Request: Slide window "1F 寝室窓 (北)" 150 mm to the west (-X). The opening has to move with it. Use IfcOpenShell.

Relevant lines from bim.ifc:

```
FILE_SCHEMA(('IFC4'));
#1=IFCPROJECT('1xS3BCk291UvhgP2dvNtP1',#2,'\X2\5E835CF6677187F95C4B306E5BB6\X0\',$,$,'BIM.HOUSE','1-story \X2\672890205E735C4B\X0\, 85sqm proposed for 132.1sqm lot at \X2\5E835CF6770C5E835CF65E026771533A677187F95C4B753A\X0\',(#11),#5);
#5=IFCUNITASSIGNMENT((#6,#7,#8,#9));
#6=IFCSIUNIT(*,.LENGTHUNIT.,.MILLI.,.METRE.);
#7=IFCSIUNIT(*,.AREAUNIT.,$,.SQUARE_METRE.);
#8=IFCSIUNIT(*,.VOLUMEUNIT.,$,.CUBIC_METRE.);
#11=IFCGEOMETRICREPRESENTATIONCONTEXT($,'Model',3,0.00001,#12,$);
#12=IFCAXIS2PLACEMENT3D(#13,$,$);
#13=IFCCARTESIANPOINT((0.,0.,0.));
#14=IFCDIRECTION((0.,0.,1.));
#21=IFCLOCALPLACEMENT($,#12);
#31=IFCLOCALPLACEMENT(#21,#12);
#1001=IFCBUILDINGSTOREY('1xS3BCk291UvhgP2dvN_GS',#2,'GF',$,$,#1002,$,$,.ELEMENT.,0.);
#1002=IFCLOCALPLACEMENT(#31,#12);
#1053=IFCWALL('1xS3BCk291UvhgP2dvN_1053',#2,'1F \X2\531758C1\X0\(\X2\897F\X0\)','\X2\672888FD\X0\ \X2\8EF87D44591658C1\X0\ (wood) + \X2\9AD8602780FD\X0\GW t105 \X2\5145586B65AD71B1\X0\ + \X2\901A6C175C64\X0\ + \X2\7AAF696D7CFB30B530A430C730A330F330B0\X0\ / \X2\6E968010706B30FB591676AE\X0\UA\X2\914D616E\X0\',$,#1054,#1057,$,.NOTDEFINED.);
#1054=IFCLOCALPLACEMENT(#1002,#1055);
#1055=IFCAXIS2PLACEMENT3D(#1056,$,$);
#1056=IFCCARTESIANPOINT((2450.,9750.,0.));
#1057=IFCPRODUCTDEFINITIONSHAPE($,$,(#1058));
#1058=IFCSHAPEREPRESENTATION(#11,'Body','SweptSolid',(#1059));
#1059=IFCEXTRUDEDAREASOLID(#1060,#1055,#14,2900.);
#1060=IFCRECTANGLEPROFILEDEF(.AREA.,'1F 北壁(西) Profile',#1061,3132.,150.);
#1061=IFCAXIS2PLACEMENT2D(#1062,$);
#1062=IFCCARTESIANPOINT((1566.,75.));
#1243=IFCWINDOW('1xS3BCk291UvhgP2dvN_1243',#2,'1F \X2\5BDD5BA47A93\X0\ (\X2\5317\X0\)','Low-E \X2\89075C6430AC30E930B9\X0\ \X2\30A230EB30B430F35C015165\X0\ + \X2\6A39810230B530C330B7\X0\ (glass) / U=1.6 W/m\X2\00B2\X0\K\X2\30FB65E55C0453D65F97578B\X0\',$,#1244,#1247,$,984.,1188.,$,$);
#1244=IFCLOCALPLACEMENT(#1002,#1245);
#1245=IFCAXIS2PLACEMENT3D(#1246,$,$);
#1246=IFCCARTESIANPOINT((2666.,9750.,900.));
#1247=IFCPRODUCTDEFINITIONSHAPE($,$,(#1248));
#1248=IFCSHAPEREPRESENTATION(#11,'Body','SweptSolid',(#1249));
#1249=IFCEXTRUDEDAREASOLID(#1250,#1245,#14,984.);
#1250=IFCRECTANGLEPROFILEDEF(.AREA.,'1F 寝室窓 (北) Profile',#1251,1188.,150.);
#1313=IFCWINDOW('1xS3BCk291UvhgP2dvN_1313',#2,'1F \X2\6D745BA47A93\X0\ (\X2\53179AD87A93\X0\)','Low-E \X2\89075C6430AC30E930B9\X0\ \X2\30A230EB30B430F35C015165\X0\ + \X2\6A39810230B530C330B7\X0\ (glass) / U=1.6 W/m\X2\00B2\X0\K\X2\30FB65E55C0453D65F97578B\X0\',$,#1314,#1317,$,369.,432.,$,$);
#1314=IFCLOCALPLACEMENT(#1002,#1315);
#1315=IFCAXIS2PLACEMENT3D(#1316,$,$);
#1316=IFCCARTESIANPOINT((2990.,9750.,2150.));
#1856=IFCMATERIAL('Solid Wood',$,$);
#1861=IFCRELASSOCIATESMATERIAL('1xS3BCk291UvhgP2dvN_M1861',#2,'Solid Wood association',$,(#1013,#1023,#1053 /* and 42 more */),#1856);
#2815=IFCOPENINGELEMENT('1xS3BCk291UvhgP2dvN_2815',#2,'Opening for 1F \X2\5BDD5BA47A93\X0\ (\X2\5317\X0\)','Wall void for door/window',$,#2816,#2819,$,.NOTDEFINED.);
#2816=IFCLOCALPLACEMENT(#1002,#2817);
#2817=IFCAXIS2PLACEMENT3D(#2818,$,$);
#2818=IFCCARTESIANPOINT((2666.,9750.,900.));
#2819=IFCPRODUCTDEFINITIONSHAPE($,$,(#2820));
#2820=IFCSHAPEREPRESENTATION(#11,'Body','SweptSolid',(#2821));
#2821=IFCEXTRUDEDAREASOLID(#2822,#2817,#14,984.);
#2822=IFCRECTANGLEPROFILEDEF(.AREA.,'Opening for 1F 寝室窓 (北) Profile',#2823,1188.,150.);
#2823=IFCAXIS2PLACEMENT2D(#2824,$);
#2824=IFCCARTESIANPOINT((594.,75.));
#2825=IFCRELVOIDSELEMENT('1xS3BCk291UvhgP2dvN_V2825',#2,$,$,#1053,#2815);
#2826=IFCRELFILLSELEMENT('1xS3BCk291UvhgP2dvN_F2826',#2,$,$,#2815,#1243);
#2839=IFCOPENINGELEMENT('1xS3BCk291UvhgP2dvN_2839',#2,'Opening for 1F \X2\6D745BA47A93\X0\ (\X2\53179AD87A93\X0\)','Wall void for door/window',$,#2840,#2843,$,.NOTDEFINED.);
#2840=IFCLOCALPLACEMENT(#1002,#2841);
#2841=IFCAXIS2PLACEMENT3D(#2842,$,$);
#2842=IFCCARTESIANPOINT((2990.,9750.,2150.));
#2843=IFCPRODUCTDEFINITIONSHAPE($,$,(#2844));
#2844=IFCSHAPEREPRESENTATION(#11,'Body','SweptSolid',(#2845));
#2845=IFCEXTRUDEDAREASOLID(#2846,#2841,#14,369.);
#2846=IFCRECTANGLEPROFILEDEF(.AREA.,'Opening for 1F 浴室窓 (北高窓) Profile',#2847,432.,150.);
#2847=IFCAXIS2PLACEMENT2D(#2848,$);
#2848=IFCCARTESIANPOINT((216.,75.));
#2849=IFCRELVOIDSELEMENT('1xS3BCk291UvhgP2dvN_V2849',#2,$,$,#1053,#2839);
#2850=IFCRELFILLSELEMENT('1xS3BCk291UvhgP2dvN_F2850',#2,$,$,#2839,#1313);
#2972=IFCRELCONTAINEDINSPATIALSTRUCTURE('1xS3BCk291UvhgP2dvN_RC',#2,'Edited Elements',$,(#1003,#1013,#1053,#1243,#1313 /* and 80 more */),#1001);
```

```python
import ifcopenshell
import ifcopenshell.api.geometry
import ifcopenshell.util.placement

model = ifcopenshell.open("bim.ifc")

window = model.by_id(1243)
opening = window.FillsVoids[0].RelatingOpeningElement
wall = opening.VoidsElements[0].RelatingBuildingElement

wall_matrix = ifcopenshell.util.placement.get_local_placement(wall.ObjectPlacement)
shift = wall_matrix[:3, 0] * -150.0
before = ifcopenshell.util.placement.get_local_placement(window.ObjectPlacement)[:3, 3].copy()

# The window is not placed relative to its opening, so move both.
for product in (opening, window):
    matrix = ifcopenshell.util.placement.get_local_placement(product.ObjectPlacement)
    matrix[:3, 3] += shift
    ifcopenshell.api.geometry.edit_object_placement(model, product=product, matrix=matrix, is_si=False)

after = ifcopenshell.util.placement.get_local_placement(window.ObjectPlacement)[:3, 3]
print("window moved by", (after - before).round(3) + 0.0)

model.write("bim_updated.ifc")
```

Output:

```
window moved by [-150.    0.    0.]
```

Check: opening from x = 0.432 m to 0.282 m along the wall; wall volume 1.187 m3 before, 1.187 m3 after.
